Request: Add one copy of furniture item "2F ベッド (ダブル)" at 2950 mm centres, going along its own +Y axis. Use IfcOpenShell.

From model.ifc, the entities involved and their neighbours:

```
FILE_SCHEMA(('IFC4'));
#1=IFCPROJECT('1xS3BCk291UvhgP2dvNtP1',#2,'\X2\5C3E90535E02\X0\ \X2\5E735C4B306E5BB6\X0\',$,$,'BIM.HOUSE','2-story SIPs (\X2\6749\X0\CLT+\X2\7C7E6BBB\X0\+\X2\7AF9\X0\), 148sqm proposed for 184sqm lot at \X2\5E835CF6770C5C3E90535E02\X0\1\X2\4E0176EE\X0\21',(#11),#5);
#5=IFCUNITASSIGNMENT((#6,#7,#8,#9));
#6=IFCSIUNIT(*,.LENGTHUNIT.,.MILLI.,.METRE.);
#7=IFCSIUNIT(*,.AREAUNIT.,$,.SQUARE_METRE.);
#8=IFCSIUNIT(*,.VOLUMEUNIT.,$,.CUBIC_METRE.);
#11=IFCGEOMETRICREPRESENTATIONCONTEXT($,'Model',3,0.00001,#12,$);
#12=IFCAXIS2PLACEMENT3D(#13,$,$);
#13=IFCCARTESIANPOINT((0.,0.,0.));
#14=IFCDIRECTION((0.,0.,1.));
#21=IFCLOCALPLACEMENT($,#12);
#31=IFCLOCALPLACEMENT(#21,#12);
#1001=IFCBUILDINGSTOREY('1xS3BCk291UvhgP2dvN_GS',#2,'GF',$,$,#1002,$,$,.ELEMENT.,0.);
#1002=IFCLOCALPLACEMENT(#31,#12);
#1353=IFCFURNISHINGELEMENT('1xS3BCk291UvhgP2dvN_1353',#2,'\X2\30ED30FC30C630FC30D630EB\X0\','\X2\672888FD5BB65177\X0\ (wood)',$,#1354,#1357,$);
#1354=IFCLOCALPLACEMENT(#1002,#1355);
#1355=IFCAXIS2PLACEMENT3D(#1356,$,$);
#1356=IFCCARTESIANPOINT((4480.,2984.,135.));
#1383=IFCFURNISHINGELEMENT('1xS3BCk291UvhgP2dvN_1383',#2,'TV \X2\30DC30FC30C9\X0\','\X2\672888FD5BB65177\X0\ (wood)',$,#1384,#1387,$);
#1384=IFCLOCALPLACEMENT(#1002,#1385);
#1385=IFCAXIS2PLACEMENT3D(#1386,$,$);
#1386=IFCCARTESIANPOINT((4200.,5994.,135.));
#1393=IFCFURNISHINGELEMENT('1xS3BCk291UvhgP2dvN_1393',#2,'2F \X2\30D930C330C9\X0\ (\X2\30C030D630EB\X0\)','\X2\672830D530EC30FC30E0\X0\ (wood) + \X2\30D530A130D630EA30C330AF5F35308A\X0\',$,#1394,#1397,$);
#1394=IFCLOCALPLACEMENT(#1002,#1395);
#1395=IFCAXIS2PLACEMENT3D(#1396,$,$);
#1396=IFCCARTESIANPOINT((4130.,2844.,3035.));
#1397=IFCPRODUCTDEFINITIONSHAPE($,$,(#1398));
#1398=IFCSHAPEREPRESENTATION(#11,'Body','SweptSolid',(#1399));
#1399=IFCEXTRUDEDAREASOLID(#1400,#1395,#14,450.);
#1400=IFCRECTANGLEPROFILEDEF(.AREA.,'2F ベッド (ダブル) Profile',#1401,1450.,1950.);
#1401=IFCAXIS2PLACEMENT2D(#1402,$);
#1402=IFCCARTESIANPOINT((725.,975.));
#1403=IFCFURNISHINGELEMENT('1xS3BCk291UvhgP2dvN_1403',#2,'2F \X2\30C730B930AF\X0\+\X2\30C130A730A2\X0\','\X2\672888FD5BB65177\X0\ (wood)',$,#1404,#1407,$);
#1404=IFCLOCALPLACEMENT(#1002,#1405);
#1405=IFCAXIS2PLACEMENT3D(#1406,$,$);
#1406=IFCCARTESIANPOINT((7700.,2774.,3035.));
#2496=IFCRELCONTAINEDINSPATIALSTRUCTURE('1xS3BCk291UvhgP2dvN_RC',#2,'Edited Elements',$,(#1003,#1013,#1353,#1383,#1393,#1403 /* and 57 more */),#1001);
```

```python
import ifcopenshell
import ifcopenshell.api.geometry
import ifcopenshell.api.root
import ifcopenshell.util.element
import ifcopenshell.util.placement
import ifcopenshell.util.unit

model = ifcopenshell.open("model.ifc")
unit_scale = ifcopenshell.util.unit.calculate_unit_scale(model)


def reuse_history(source, copy):
    """copy_class also copies each property set's owner history, people and application; keep the originals."""
    for rel in copy.IsDefinedBy:
        if rel.is_a("IfcRelDefinesByProperties") and (history := rel.RelatingPropertyDefinition.OwnerHistory):
            rel.RelatingPropertyDefinition.OwnerHistory = source.OwnerHistory
            ifcopenshell.util.element.remove_deep2(model, history)


source = model.by_guid("1xS3BCk291UvhgP2dvN_1393")
base = ifcopenshell.util.placement.get_local_placement(source.ObjectPlacement)
step = base[:3, 1] * 2.95 / unit_scale

for i in range(1, 2):
    copy = ifcopenshell.api.root.copy_class(model, product=source)
    copy.Representation = ifcopenshell.util.element.copy_deep(
        model, source.Representation, exclude=["IfcGeometricRepresentationContext", "IfcRepresentationMap"]
    )
    reuse_history(source, copy)
    matrix = base.copy()
    matrix[:3, 3] += i * step
    print("added at", matrix[:3, 3].round(3) + 0.0)
    ifcopenshell.api.geometry.edit_object_placement(model, product=copy, matrix=matrix, is_si=False)

model.write("model_updated.ifc")
```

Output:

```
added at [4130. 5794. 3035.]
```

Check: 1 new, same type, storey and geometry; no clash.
